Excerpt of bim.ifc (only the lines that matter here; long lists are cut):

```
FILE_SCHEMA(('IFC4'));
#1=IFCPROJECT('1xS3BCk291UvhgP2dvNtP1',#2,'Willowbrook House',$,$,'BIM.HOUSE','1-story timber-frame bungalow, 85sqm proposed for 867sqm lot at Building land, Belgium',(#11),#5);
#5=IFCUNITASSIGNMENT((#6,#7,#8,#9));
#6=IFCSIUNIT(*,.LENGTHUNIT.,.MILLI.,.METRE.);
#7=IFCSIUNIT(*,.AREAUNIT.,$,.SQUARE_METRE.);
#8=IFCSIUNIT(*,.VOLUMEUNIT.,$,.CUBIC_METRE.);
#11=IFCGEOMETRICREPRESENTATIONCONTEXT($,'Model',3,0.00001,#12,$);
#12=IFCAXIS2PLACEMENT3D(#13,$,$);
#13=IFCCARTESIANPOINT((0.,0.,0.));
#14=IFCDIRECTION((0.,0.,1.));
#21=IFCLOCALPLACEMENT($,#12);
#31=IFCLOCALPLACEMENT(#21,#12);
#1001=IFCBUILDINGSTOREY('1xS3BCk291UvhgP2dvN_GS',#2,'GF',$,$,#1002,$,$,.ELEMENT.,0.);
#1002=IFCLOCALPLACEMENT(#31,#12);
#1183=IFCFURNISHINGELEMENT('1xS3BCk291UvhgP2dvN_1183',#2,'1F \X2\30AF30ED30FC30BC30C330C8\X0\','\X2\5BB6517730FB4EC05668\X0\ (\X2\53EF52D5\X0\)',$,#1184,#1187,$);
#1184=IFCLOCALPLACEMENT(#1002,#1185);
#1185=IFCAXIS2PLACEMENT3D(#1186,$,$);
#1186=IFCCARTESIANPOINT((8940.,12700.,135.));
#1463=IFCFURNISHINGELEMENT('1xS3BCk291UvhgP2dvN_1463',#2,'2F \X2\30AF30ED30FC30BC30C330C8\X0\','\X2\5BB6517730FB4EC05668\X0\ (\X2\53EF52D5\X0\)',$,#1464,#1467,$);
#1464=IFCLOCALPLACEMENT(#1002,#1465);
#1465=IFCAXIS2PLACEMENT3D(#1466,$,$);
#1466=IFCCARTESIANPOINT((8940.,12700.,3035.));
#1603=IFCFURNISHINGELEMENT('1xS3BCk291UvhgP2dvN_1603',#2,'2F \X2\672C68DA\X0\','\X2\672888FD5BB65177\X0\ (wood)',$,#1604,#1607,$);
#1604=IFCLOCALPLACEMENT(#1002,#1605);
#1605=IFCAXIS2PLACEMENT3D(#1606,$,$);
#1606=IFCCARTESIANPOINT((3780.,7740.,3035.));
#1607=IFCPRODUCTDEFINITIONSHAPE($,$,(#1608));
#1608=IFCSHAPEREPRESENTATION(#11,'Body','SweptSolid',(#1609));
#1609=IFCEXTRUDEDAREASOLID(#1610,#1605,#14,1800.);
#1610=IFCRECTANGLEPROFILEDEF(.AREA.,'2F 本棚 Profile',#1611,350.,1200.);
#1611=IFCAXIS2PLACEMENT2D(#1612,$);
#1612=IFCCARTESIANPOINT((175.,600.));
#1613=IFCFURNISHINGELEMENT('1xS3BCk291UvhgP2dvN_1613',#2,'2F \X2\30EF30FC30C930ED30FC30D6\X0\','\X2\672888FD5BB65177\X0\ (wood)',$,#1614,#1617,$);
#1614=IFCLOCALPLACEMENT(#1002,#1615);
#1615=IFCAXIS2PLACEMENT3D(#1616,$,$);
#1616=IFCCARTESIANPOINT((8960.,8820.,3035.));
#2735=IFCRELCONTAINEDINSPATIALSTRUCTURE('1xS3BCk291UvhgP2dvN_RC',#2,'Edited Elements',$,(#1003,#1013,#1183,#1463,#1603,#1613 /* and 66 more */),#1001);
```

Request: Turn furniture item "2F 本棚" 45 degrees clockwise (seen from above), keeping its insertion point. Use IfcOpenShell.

```python
import ifcopenshell
import ifcopenshell.api.geometry
import ifcopenshell.util.placement

model = ifcopenshell.open("bim.ifc")

item = model.by_guid("1xS3BCk291UvhgP2dvN_1603")
matrix = ifcopenshell.util.placement.get_local_placement(item.ObjectPlacement)
matrix = matrix @ ifcopenshell.util.placement.rotation(-45, "Z")
ifcopenshell.api.geometry.edit_object_placement(model, product=item, matrix=matrix, is_si=False)

print(ifcopenshell.util.placement.get_local_placement(item.ObjectPlacement).round(3) + 0.0)

model.write("bim_edited.ifc")
```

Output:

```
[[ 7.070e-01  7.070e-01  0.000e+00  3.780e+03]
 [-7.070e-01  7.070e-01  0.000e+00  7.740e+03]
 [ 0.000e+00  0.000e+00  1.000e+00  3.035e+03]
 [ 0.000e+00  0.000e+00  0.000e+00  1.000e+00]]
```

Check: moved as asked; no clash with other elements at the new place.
